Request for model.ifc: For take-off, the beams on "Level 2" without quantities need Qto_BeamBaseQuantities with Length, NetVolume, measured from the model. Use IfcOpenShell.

First a look at what the model holds.

```python
import ifcopenshell
import ifcopenshell.util.element
import ifcopenshell.util.unit

model = ifcopenshell.open("model.ifc")
print(model.schema)
for unit_type in ("LENGTHUNIT", "AREAUNIT", "VOLUMEUNIT"):
    print(unit_type, ifcopenshell.util.unit.calculate_unit_scale(model, unit_type))
storey = next(s for s in model.by_type("IfcBuildingStorey") if s.Name == "Level 2")
beams = [e for e in ifcopenshell.util.element.get_decomposition(storey) if e.is_a("IfcBeam")]
for e in sorted(beams, key=lambda e: e.id()):
    print(e.id(), e.is_a(), e.Name, list(ifcopenshell.util.element.get_psets(e, qtos_only=True)), sep=" | ")
```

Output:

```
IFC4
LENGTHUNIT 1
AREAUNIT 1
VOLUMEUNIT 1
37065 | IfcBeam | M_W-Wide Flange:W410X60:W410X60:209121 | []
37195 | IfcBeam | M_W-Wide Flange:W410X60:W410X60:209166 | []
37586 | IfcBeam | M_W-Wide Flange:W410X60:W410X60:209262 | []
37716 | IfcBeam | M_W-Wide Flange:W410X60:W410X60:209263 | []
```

```python
import ifcopenshell
import ifcopenshell.api.pset
import ifcopenshell.geom
import ifcopenshell.util.element
import ifcopenshell.util.shape
import ifcopenshell.util.unit

model = ifcopenshell.open("model.ifc")
unit_scale = ifcopenshell.util.unit.calculate_unit_scale(model)
volume_scale = ifcopenshell.util.unit.calculate_unit_scale(model, "VOLUMEUNIT")
settings = ifcopenshell.geom.settings()

storey = next(s for s in model.by_type("IfcBuildingStorey") if s.Name == "Level 2")
beams = [e for e in ifcopenshell.util.element.get_decomposition(storey) if e.is_a("IfcBeam")]

for e in sorted(beams, key=lambda e: e.id()):
    if ifcopenshell.util.element.get_psets(e, qtos_only=True, should_inherit=False):
        continue
    # Geometry comes back in metres, in the element's own axes.
    shape = ifcopenshell.geom.create_shape(settings, e)
    values = {
        "Length": ifcopenshell.util.shape.get_max_xyz(shape.geometry) / unit_scale,
        "NetVolume": ifcopenshell.util.shape.get_volume(shape.geometry) / volume_scale,
    }
    qto = ifcopenshell.api.pset.add_qto(model, product=e, name="Qto_BeamBaseQuantities")
    ifcopenshell.api.pset.edit_qto(model, qto=qto, properties=values)
    print(e.id(), {k: round(v, 3) for k, v in values.items()})

model.write("model_edited.ifc")
```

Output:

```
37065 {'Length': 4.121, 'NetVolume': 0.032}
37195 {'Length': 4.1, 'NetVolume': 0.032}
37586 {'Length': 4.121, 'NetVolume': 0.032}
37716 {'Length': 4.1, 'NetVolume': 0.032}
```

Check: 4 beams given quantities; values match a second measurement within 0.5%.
